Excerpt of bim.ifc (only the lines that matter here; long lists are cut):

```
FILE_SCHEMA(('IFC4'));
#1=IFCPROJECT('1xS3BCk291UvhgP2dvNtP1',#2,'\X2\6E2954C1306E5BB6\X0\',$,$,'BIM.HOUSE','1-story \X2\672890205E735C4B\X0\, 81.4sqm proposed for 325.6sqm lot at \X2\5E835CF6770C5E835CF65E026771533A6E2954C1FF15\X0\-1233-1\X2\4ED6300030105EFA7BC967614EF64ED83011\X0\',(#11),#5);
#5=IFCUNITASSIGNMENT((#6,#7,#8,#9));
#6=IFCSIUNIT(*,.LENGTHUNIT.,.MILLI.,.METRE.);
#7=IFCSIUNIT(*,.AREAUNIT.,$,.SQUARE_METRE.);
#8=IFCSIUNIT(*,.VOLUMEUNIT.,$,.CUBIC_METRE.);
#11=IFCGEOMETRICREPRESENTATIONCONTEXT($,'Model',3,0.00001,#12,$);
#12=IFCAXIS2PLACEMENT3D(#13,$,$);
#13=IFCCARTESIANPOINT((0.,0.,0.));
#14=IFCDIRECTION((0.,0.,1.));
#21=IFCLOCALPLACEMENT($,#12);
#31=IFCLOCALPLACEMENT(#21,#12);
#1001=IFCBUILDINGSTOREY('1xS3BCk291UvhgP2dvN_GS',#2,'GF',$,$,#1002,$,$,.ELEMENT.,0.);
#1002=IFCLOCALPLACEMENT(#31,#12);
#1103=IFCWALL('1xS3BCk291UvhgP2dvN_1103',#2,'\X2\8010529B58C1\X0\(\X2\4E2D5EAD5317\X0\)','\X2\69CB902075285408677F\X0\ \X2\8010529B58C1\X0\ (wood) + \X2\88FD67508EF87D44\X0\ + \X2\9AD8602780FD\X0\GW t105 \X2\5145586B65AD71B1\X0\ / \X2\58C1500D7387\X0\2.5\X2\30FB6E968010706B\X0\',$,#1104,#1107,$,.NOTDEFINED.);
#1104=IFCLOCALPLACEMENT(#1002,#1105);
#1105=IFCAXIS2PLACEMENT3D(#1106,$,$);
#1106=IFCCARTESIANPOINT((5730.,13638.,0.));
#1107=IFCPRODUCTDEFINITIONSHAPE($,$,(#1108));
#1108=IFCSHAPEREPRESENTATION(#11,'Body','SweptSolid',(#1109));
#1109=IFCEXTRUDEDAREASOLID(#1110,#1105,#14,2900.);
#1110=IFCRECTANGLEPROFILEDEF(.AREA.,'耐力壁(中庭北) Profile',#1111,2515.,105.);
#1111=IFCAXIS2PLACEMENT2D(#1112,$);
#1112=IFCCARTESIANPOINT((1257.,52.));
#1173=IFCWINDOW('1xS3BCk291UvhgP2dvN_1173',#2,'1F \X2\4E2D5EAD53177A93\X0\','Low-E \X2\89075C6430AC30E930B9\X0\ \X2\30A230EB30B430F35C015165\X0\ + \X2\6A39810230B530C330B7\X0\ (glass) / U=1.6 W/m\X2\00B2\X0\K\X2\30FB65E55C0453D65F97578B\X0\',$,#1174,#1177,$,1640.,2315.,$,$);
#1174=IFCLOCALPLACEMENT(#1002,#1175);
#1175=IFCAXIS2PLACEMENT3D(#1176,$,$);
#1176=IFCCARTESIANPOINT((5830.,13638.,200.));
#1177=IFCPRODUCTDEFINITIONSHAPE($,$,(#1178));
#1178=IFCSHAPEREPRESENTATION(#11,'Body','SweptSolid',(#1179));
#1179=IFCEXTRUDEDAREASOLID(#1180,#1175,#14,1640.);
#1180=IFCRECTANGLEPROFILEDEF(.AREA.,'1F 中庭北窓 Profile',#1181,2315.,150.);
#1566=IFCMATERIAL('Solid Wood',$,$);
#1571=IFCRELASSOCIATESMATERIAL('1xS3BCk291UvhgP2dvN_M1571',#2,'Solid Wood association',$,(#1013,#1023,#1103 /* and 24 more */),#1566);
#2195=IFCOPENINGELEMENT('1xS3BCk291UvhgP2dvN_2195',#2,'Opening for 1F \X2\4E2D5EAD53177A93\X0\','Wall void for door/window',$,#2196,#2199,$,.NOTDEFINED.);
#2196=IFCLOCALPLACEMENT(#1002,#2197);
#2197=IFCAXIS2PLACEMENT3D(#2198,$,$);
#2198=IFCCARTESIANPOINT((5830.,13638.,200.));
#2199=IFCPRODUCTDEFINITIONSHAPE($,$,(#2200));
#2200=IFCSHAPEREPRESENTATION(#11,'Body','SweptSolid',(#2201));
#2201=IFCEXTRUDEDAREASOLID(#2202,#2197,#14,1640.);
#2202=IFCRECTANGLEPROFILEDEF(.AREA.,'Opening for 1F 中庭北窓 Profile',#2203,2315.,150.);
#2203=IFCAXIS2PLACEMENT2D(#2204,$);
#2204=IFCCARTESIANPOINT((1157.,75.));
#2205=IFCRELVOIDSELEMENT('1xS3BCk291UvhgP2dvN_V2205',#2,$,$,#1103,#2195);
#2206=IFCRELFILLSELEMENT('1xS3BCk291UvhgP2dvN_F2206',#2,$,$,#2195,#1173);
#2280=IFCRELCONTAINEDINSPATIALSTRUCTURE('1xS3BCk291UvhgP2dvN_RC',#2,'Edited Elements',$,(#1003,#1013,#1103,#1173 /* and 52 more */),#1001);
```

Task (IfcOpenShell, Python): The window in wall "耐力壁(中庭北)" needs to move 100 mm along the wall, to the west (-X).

```python
import ifcopenshell
import ifcopenshell.api.geometry
import ifcopenshell.util.placement
import ifcopenshell.util.unit

model = ifcopenshell.open("bim.ifc")
unit_scale = ifcopenshell.util.unit.calculate_unit_scale(model)

window = model.by_guid("1xS3BCk291UvhgP2dvN_1173")
opening = window.FillsVoids[0].RelatingOpeningElement
wall = opening.VoidsElements[0].RelatingBuildingElement

wall_matrix = ifcopenshell.util.placement.get_local_placement(wall.ObjectPlacement)
shift = wall_matrix[:3, 0] * -0.1 / unit_scale
before = ifcopenshell.util.placement.get_local_placement(window.ObjectPlacement)[:3, 3].copy()

# The window is not placed relative to its opening, so move both.
for product in (opening, window):
    matrix = ifcopenshell.util.placement.get_local_placement(product.ObjectPlacement)
    matrix[:3, 3] += shift
    ifcopenshell.api.geometry.edit_object_placement(model, product=product, matrix=matrix, is_si=False)

after = ifcopenshell.util.placement.get_local_placement(window.ObjectPlacement)[:3, 3]
print("window moved by", (after - before).round(3) + 0.0)

model.write("bim-out.ifc")
```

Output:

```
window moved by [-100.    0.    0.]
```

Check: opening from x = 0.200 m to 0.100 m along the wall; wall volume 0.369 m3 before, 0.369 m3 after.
